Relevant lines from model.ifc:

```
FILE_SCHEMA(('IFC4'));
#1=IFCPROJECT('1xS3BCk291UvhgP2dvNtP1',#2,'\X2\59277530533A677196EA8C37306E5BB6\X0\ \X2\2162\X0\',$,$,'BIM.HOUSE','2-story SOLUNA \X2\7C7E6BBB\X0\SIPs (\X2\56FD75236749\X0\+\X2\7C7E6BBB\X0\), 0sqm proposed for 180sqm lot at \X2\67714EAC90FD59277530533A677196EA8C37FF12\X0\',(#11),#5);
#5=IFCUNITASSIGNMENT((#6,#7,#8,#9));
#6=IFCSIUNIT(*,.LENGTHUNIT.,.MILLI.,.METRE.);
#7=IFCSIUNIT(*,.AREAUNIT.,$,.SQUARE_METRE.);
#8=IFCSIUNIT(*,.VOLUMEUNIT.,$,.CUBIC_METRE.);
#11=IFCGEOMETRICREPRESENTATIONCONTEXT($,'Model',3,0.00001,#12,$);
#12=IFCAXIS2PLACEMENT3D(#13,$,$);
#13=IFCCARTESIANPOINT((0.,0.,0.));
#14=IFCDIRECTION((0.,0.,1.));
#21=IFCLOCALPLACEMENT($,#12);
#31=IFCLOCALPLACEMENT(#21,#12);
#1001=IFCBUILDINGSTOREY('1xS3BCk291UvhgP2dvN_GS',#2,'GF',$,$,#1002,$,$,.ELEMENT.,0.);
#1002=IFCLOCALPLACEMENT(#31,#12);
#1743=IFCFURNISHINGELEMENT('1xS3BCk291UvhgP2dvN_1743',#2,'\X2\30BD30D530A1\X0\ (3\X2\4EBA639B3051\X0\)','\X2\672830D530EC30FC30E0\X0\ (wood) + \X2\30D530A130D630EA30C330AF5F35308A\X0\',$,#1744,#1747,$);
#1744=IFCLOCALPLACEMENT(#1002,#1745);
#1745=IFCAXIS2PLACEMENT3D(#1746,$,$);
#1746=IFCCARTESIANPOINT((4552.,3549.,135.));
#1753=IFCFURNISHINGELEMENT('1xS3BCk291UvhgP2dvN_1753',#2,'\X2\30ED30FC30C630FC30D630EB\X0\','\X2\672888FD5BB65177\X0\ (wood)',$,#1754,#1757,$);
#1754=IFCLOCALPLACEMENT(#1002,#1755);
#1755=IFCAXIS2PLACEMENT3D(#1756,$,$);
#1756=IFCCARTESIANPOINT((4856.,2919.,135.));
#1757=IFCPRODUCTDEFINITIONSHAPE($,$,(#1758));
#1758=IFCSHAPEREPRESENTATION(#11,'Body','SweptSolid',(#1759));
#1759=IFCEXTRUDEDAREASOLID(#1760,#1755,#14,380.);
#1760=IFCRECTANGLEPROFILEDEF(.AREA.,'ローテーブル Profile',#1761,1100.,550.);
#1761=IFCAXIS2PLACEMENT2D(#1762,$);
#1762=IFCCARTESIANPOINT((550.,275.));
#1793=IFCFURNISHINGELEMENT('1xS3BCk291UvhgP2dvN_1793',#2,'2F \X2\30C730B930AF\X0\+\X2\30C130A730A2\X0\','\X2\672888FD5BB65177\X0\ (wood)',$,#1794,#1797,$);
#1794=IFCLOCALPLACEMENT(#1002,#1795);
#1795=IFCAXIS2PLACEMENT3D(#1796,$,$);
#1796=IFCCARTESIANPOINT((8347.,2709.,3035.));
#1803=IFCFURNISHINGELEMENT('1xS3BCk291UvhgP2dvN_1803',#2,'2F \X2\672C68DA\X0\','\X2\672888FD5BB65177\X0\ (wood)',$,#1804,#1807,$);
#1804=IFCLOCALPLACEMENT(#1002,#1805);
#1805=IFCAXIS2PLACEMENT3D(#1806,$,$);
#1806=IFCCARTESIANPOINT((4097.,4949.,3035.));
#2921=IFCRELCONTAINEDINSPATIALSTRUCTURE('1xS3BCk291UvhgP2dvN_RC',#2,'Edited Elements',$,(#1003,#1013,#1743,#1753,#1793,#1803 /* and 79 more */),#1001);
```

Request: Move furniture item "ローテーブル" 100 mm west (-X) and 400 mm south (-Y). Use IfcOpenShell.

```python
import ifcopenshell
import ifcopenshell.api.geometry
import ifcopenshell.util.placement
import ifcopenshell.util.unit

model = ifcopenshell.open("model.ifc")
unit_scale = ifcopenshell.util.unit.calculate_unit_scale(model)

item = model.by_id(1753)
matrix = ifcopenshell.util.placement.get_local_placement(item.ObjectPlacement)
matrix[0, 3] -= 0.1 / unit_scale
matrix[1, 3] -= 0.4 / unit_scale
ifcopenshell.api.geometry.edit_object_placement(model, product=item, matrix=matrix, is_si=False)

print(ifcopenshell.util.placement.get_local_placement(item.ObjectPlacement).round(3) + 0.0)

model.write("model_edited.ifc")
```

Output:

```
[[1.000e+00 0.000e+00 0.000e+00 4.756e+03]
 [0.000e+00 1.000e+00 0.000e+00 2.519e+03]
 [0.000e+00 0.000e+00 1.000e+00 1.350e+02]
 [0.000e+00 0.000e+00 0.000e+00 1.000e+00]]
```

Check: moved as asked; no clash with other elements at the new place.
